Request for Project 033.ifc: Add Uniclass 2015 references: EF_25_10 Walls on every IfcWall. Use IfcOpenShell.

First a look at what the model holds.

```python
import ifcopenshell

model = ifcopenshell.open("Project 033.ifc")
print(model.schema)
print("classifications:", [c.Name for c in model.by_type("IfcClassification")])
for ifc_class in ("IfcDoor", "IfcRoof", "IfcStair", "IfcWall", "IfcWindow"):
    print(ifc_class, len(model.by_type(ifc_class)))
```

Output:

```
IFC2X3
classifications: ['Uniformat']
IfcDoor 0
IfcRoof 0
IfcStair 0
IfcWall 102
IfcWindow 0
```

```python
import ifcopenshell
import ifcopenshell.api.classification

model = ifcopenshell.open("Project 033.ifc")

# IFC2X3 requires Source and Edition and has no link from the project to the system.
system = model.create_entity("IfcClassification", Source="NBS", Edition="2015", Name="Uniclass 2015")

codes = {
    "IfcWall": ("EF_25_10", "Walls"),
}
for ifc_class, (code, name) in codes.items():
    products = model.by_type(ifc_class)
    ifcopenshell.api.classification.add_reference(
        model, products=products, classification=system, identification=code, name=name
    )
    print(code, len(products))

model.write("Project 033-out.ifc")
```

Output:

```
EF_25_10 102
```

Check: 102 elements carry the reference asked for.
